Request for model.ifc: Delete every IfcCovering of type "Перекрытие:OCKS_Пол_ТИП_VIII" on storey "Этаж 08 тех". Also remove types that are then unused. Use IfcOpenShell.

First a look at what the model holds.

```python
import ifcopenshell
import ifcopenshell.util.element

model = ifcopenshell.open("model.ifc")
print(model.schema)
storey = next(s for s in model.by_type("IfcBuildingStorey") if s.Name == "Этаж 08 тех")
coverings = [e for e in ifcopenshell.util.element.get_decomposition(storey) if e.is_a("IfcCovering")]
seen = {}
for e in coverings:
    element_type = ifcopenshell.util.element.get_type(e)
    name = element_type.Name if element_type not in (None, e) else None
    seen[name] = seen.get(name, 0) + 1
for name, count in sorted(seen.items(), key=str):
    print(count, "x", name)
```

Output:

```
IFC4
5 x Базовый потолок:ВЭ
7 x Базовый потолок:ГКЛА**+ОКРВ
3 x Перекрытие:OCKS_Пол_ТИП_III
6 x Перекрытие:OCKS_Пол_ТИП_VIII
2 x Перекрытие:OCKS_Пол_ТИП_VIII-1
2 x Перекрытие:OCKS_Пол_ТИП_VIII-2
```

```python
import ifcopenshell
import ifcopenshell.api.root
import ifcopenshell.util.element

model = ifcopenshell.open("model.ifc")

storey = next(s for s in model.by_type("IfcBuildingStorey") if s.Name == "Этаж 08 тех")
coverings = [e for e in ifcopenshell.util.element.get_decomposition(storey) if e.is_a("IfcCovering")]
targets = [e for e in coverings if (t := ifcopenshell.util.element.get_type(e)) not in (None, e) and t.Name == "Перекрытие:OCKS_Пол_ТИП_VIII"]
types = {ifcopenshell.util.element.get_type(e) for e in targets} - {None, *targets}

for e in targets:
    ifcopenshell.api.root.remove_product(model, product=e)
print(len(targets), "removed")

unused = [t for t in types if not ifcopenshell.util.element.get_types(t)]
for t in unused:
    ifcopenshell.api.root.remove_product(model, product=t)
print(len(unused), "unused types removed")

model.write("model_rev.ifc")
```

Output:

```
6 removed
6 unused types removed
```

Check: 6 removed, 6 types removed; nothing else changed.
